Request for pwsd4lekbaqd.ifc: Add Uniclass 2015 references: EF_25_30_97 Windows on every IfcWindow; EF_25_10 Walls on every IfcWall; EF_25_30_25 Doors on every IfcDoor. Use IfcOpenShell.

First a look at what the model holds.

```python
import ifcopenshell

model = ifcopenshell.open("pwsd4lekbaqd.ifc")
print(model.schema)
print("classifications:", [c.Name for c in model.by_type("IfcClassification")])
for ifc_class in ("IfcDoor", "IfcRoof", "IfcStair", "IfcWall", "IfcWindow"):
    print(ifc_class, len(model.by_type(ifc_class)))
```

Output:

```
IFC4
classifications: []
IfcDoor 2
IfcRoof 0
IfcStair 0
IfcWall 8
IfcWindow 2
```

```python
import ifcopenshell
import ifcopenshell.api.classification

model = ifcopenshell.open("pwsd4lekbaqd.ifc")

system = ifcopenshell.api.classification.add_classification(model, classification="Uniclass 2015")

codes = {
    "IfcWindow": ("EF_25_30_97", "Windows"),
    "IfcWall": ("EF_25_10", "Walls"),
    "IfcDoor": ("EF_25_30_25", "Doors"),
}
for ifc_class, (code, name) in codes.items():
    products = model.by_type(ifc_class)
    ifcopenshell.api.classification.add_reference(
        model, products=products, classification=system, identification=code, name=name
    )
    print(code, len(products))

model.write("pwsd4lekbaqd-out.ifc")
```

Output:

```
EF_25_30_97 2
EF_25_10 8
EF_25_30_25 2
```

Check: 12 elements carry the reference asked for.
